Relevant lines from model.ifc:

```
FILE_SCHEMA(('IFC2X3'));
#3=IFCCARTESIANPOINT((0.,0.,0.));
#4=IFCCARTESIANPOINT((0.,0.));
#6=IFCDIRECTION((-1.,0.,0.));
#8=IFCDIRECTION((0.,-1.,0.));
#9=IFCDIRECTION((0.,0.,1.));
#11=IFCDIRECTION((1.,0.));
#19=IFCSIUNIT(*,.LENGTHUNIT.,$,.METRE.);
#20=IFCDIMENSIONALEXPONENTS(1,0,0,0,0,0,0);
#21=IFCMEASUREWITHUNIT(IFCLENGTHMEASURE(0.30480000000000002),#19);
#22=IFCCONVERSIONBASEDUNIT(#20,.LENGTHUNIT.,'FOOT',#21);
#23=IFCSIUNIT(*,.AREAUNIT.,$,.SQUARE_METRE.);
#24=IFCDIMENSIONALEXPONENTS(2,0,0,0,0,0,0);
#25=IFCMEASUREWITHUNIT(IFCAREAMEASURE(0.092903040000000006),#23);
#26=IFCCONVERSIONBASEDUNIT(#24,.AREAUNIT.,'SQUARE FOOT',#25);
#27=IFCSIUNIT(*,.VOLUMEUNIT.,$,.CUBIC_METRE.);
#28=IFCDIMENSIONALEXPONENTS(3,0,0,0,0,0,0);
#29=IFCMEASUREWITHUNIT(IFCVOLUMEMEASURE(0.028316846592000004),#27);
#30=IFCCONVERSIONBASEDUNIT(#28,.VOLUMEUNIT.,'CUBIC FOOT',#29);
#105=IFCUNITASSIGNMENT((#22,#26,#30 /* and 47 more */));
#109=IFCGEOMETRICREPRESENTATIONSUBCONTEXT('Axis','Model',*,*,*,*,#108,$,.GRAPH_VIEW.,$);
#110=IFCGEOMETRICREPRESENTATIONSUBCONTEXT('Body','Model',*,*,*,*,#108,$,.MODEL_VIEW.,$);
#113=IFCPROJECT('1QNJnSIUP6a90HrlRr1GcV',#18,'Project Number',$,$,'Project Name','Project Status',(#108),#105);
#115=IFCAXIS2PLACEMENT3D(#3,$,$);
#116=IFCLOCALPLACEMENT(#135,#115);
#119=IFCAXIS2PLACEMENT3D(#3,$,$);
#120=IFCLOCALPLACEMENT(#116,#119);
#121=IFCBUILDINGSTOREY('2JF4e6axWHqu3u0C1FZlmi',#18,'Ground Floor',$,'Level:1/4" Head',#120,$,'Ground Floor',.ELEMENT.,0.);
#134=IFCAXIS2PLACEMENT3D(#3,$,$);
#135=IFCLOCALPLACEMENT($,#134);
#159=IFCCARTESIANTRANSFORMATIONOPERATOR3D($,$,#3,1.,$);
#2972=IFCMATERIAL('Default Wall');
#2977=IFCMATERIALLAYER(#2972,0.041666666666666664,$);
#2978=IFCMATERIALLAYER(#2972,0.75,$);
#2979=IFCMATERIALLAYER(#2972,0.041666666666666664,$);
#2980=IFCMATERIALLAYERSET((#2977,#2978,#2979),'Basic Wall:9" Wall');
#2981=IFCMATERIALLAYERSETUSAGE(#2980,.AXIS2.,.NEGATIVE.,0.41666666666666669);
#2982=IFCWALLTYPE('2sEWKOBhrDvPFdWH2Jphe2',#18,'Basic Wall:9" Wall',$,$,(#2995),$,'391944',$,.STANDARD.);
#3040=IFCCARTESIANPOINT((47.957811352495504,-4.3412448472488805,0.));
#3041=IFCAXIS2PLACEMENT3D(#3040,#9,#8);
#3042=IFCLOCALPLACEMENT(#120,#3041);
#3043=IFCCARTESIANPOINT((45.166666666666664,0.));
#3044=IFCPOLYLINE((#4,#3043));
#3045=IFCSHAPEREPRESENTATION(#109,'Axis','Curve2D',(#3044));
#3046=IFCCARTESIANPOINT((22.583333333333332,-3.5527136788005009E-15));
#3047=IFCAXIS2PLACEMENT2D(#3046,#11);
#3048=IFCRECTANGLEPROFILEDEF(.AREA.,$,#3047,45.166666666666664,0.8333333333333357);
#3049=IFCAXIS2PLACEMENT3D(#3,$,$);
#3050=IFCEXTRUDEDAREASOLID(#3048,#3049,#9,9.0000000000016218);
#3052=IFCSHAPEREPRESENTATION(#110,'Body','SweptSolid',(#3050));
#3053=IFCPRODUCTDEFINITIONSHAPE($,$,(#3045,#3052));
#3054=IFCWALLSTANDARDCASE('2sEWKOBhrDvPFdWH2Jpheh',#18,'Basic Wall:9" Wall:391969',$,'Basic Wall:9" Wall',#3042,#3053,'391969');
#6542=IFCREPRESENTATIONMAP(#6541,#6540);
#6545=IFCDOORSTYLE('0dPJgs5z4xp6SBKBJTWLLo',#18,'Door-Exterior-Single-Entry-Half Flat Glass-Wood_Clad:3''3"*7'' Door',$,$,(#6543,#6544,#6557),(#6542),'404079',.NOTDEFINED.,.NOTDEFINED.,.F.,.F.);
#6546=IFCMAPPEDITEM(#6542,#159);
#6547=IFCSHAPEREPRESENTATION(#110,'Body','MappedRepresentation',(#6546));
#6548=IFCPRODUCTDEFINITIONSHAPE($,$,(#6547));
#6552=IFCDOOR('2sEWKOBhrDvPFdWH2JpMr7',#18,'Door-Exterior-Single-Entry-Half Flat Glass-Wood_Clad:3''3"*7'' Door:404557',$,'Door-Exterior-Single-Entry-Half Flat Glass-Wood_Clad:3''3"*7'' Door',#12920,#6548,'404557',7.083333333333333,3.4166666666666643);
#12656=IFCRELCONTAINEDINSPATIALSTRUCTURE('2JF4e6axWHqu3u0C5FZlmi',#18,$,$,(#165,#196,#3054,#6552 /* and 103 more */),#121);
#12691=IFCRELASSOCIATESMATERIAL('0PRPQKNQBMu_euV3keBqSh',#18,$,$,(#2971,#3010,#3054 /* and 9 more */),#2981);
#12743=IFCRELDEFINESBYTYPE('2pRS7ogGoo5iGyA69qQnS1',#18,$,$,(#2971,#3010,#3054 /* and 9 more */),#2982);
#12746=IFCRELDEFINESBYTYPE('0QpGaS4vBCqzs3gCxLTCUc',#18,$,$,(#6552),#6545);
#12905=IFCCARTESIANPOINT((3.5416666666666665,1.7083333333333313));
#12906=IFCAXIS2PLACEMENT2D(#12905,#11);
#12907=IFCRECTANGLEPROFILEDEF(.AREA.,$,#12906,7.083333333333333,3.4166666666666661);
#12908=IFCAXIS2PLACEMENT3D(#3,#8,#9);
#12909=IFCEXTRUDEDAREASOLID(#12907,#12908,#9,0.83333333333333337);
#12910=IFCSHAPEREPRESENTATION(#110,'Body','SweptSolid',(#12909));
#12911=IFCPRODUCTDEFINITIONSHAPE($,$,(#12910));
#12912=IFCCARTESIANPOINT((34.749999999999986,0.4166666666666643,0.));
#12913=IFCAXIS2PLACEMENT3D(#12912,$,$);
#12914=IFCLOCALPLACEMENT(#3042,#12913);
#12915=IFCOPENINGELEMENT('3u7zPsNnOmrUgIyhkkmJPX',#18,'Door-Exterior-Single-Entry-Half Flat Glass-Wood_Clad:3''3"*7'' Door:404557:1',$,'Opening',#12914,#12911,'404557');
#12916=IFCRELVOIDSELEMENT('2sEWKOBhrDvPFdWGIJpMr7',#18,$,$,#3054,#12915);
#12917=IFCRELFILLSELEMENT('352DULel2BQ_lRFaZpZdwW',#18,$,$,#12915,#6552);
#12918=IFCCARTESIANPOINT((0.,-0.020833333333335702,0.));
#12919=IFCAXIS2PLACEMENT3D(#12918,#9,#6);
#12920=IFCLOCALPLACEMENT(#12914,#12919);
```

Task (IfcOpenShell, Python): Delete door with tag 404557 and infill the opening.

```python
import ifcopenshell
import ifcopenshell.api.feature
import ifcopenshell.api.root
import ifcopenshell.geom
import ifcopenshell.util.shape

model = ifcopenshell.open("model.ifc")
settings = ifcopenshell.geom.settings()


def volume(element):
    """Net volume in cubic metres, openings subtracted."""
    shape = ifcopenshell.geom.create_shape(settings, element)
    return ifcopenshell.util.shape.get_volume(shape.geometry)


door = model.by_guid("2sEWKOBhrDvPFdWH2JpMr7")
opening = door.FillsVoids[0].RelatingOpeningElement
wall = opening.VoidsElements[0].RelatingBuildingElement
before = volume(wall)

ifcopenshell.api.root.remove_product(model, product=door)
ifcopenshell.api.feature.remove_feature(model, feature=opening)

after = volume(wall)

print(f"wall volume {before:.3f} -> {after:.3f} m3")

model.write("model-out.ifc")
```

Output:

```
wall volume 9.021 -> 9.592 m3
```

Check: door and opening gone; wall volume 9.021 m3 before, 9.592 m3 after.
